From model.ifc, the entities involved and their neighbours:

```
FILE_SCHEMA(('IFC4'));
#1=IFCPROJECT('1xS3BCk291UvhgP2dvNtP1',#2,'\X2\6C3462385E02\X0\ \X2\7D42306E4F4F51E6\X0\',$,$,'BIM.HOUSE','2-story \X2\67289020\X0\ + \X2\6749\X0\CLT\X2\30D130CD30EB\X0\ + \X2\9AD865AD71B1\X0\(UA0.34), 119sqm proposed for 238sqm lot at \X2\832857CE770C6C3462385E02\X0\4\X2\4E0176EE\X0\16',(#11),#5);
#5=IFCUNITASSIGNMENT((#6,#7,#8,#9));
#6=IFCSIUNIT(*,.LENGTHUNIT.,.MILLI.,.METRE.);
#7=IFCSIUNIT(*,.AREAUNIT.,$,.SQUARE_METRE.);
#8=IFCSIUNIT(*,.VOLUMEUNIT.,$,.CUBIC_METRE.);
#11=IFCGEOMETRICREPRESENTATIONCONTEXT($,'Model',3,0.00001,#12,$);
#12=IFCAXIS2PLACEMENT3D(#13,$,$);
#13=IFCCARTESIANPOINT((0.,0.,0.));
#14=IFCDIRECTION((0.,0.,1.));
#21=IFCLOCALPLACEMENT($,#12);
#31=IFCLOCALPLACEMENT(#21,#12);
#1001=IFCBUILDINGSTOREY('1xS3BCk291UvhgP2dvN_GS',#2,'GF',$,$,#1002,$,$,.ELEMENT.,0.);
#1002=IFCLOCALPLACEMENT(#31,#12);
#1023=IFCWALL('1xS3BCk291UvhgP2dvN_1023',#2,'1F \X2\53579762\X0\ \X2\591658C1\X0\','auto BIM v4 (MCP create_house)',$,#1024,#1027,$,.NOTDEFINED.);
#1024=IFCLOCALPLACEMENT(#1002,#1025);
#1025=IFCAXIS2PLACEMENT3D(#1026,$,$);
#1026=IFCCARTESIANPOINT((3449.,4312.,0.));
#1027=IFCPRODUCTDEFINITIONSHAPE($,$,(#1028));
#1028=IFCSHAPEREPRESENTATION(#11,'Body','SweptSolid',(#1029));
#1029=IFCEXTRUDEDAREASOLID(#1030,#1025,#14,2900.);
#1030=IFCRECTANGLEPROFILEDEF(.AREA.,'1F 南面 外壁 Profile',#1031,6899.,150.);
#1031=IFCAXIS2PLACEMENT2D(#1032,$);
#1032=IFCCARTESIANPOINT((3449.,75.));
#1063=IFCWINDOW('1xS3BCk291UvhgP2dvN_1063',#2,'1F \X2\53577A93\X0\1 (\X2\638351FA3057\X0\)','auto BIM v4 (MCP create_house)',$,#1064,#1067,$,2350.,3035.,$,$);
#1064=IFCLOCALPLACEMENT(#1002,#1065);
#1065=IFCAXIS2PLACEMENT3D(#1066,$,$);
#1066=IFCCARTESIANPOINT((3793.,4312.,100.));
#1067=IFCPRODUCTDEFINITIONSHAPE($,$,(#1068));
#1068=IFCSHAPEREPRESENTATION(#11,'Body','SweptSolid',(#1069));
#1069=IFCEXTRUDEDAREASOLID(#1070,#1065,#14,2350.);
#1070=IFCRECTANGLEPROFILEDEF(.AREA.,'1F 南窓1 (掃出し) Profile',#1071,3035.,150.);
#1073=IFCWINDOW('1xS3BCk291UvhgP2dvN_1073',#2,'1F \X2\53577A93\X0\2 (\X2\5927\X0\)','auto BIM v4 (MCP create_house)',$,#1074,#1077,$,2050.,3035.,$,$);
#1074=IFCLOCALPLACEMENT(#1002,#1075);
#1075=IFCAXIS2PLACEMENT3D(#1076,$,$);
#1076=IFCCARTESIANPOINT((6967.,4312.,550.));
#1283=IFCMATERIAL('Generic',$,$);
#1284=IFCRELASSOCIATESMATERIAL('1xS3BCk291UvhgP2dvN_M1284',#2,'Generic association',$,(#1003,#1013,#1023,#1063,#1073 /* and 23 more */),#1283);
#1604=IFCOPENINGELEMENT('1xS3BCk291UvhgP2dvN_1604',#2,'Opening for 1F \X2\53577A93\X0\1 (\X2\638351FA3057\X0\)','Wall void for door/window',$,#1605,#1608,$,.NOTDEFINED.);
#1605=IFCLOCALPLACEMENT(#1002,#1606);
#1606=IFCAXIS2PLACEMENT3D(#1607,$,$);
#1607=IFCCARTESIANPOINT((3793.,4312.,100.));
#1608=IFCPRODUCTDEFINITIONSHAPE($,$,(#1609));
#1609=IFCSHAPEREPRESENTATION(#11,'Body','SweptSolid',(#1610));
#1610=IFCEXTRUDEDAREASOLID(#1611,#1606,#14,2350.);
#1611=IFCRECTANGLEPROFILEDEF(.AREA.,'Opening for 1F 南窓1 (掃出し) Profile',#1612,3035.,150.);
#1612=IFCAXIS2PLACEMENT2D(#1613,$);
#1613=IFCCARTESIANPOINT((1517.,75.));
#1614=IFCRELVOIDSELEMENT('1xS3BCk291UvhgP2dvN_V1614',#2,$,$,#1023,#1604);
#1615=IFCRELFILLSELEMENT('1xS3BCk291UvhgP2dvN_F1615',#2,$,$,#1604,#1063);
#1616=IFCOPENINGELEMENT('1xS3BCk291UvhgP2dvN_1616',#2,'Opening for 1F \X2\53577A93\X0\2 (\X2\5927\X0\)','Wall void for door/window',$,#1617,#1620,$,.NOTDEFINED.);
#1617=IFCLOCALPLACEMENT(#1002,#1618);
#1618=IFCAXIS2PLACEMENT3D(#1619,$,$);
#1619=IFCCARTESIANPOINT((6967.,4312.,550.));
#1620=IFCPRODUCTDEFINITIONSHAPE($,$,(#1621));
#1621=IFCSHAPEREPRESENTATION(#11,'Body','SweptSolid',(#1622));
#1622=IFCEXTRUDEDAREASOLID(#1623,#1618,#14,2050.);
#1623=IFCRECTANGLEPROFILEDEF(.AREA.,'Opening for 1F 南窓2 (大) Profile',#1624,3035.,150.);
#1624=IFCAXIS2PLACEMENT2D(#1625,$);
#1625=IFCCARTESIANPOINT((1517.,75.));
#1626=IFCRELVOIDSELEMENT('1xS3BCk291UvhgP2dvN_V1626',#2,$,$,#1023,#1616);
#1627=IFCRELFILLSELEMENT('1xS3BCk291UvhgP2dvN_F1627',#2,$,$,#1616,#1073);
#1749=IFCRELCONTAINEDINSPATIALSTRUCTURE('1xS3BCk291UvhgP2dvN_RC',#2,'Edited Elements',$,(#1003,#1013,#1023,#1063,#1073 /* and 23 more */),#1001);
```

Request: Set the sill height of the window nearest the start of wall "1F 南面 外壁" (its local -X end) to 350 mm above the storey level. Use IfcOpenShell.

```python
import numpy as np
import ifcopenshell
import ifcopenshell.api.geometry
import ifcopenshell.geom
import ifcopenshell.util.element
import ifcopenshell.util.placement
import ifcopenshell.util.shape
import ifcopenshell.util.unit

model = ifcopenshell.open("model.ifc")
unit_scale = ifcopenshell.util.unit.calculate_unit_scale(model)

window = model.by_id(1063)
opening = window.FillsVoids[0].RelatingOpeningElement
storey = ifcopenshell.util.element.get_container(window, ifc_class="IfcBuildingStorey")
level = ifcopenshell.util.placement.get_local_placement(storey.ObjectPlacement)[2, 3]

# The opening's origin need not be at the sill, so measure its lowest point.
shape = ifcopenshell.geom.create_shape(ifcopenshell.geom.settings(), opening)
bottom = ifcopenshell.util.shape.get_shape_bottom_elevation(shape, shape.geometry) / unit_scale
dz = level + 0.35 / unit_scale - bottom

shift = np.array([0.0, 0.0, dz])
# The window is not placed relative to its opening, so move both.
for product in (opening, window):
    matrix = ifcopenshell.util.placement.get_local_placement(product.ObjectPlacement)
    matrix[:3, 3] += shift
    ifcopenshell.api.geometry.edit_object_placement(model, product=product, matrix=matrix, is_si=False)

print(f"moved by {dz * unit_scale:+.3f} m")

model.write("model_updated.ifc")
```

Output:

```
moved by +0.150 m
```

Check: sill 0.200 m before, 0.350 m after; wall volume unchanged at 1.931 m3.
